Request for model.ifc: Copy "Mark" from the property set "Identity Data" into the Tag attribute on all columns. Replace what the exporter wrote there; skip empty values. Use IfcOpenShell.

First a look at what the model holds.

```python
import ifcopenshell
import ifcopenshell.util.element

model = ifcopenshell.open("model.ifc")
print(model.schema)
columns = model.by_type("IfcColumn")
print(len(columns), "columns")
for e in columns[:8]:
    source = ifcopenshell.util.element.get_pset(e, "Identity Data", "Mark")
    target = e.Tag
    print(e.id(), repr(source), repr(target), sep=" | ")
```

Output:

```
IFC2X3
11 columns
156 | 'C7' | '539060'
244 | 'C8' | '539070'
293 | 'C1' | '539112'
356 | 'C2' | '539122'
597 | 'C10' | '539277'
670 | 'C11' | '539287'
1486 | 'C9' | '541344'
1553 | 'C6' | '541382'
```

```python
import ifcopenshell
import ifcopenshell.util.element

model = ifcopenshell.open("model.ifc")

count = 0
for e in model.by_type("IfcColumn"):
    value = ifcopenshell.util.element.get_pset(e, "Identity Data", "Mark")
    current = e.Tag
    if not value or not value.strip() or current == value:
        continue
    e.Tag = value
    count += 1

print(count, "columns updated")

model.write("model_v2.ifc")
```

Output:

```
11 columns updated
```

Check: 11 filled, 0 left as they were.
